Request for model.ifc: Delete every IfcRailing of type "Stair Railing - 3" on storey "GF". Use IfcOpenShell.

First a look at what the model holds.

```python
import ifcopenshell
import ifcopenshell.util.element

model = ifcopenshell.open("model.ifc")
print(model.schema)
storey = next(s for s in model.by_type("IfcBuildingStorey") if s.Name == "GF")
railings = [e for e in ifcopenshell.util.element.get_decomposition(storey) if e.is_a("IfcRailing")]
seen = {}
for e in railings:
    element_type = ifcopenshell.util.element.get_type(e)
    name = element_type.Name if element_type not in (None, e) else None
    seen[name] = seen.get(name, 0) + 1
for name, count in sorted(seen.items(), key=str):
    print(count, "x", name)
```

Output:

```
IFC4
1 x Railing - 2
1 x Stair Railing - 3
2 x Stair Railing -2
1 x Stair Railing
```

```python
import ifcopenshell
import ifcopenshell.api.root
import ifcopenshell.util.element

model = ifcopenshell.open("model.ifc")

storey = next(s for s in model.by_type("IfcBuildingStorey") if s.Name == "GF")
railings = [e for e in ifcopenshell.util.element.get_decomposition(storey) if e.is_a("IfcRailing")]
targets = [e for e in railings if (t := ifcopenshell.util.element.get_type(e)) not in (None, e) and t.Name == "Stair Railing - 3"]

for e in targets:
    ifcopenshell.api.root.remove_product(model, product=e)
print(len(targets), "removed")

model.write("model-out.ifc")
```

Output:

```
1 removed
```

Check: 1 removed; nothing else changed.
